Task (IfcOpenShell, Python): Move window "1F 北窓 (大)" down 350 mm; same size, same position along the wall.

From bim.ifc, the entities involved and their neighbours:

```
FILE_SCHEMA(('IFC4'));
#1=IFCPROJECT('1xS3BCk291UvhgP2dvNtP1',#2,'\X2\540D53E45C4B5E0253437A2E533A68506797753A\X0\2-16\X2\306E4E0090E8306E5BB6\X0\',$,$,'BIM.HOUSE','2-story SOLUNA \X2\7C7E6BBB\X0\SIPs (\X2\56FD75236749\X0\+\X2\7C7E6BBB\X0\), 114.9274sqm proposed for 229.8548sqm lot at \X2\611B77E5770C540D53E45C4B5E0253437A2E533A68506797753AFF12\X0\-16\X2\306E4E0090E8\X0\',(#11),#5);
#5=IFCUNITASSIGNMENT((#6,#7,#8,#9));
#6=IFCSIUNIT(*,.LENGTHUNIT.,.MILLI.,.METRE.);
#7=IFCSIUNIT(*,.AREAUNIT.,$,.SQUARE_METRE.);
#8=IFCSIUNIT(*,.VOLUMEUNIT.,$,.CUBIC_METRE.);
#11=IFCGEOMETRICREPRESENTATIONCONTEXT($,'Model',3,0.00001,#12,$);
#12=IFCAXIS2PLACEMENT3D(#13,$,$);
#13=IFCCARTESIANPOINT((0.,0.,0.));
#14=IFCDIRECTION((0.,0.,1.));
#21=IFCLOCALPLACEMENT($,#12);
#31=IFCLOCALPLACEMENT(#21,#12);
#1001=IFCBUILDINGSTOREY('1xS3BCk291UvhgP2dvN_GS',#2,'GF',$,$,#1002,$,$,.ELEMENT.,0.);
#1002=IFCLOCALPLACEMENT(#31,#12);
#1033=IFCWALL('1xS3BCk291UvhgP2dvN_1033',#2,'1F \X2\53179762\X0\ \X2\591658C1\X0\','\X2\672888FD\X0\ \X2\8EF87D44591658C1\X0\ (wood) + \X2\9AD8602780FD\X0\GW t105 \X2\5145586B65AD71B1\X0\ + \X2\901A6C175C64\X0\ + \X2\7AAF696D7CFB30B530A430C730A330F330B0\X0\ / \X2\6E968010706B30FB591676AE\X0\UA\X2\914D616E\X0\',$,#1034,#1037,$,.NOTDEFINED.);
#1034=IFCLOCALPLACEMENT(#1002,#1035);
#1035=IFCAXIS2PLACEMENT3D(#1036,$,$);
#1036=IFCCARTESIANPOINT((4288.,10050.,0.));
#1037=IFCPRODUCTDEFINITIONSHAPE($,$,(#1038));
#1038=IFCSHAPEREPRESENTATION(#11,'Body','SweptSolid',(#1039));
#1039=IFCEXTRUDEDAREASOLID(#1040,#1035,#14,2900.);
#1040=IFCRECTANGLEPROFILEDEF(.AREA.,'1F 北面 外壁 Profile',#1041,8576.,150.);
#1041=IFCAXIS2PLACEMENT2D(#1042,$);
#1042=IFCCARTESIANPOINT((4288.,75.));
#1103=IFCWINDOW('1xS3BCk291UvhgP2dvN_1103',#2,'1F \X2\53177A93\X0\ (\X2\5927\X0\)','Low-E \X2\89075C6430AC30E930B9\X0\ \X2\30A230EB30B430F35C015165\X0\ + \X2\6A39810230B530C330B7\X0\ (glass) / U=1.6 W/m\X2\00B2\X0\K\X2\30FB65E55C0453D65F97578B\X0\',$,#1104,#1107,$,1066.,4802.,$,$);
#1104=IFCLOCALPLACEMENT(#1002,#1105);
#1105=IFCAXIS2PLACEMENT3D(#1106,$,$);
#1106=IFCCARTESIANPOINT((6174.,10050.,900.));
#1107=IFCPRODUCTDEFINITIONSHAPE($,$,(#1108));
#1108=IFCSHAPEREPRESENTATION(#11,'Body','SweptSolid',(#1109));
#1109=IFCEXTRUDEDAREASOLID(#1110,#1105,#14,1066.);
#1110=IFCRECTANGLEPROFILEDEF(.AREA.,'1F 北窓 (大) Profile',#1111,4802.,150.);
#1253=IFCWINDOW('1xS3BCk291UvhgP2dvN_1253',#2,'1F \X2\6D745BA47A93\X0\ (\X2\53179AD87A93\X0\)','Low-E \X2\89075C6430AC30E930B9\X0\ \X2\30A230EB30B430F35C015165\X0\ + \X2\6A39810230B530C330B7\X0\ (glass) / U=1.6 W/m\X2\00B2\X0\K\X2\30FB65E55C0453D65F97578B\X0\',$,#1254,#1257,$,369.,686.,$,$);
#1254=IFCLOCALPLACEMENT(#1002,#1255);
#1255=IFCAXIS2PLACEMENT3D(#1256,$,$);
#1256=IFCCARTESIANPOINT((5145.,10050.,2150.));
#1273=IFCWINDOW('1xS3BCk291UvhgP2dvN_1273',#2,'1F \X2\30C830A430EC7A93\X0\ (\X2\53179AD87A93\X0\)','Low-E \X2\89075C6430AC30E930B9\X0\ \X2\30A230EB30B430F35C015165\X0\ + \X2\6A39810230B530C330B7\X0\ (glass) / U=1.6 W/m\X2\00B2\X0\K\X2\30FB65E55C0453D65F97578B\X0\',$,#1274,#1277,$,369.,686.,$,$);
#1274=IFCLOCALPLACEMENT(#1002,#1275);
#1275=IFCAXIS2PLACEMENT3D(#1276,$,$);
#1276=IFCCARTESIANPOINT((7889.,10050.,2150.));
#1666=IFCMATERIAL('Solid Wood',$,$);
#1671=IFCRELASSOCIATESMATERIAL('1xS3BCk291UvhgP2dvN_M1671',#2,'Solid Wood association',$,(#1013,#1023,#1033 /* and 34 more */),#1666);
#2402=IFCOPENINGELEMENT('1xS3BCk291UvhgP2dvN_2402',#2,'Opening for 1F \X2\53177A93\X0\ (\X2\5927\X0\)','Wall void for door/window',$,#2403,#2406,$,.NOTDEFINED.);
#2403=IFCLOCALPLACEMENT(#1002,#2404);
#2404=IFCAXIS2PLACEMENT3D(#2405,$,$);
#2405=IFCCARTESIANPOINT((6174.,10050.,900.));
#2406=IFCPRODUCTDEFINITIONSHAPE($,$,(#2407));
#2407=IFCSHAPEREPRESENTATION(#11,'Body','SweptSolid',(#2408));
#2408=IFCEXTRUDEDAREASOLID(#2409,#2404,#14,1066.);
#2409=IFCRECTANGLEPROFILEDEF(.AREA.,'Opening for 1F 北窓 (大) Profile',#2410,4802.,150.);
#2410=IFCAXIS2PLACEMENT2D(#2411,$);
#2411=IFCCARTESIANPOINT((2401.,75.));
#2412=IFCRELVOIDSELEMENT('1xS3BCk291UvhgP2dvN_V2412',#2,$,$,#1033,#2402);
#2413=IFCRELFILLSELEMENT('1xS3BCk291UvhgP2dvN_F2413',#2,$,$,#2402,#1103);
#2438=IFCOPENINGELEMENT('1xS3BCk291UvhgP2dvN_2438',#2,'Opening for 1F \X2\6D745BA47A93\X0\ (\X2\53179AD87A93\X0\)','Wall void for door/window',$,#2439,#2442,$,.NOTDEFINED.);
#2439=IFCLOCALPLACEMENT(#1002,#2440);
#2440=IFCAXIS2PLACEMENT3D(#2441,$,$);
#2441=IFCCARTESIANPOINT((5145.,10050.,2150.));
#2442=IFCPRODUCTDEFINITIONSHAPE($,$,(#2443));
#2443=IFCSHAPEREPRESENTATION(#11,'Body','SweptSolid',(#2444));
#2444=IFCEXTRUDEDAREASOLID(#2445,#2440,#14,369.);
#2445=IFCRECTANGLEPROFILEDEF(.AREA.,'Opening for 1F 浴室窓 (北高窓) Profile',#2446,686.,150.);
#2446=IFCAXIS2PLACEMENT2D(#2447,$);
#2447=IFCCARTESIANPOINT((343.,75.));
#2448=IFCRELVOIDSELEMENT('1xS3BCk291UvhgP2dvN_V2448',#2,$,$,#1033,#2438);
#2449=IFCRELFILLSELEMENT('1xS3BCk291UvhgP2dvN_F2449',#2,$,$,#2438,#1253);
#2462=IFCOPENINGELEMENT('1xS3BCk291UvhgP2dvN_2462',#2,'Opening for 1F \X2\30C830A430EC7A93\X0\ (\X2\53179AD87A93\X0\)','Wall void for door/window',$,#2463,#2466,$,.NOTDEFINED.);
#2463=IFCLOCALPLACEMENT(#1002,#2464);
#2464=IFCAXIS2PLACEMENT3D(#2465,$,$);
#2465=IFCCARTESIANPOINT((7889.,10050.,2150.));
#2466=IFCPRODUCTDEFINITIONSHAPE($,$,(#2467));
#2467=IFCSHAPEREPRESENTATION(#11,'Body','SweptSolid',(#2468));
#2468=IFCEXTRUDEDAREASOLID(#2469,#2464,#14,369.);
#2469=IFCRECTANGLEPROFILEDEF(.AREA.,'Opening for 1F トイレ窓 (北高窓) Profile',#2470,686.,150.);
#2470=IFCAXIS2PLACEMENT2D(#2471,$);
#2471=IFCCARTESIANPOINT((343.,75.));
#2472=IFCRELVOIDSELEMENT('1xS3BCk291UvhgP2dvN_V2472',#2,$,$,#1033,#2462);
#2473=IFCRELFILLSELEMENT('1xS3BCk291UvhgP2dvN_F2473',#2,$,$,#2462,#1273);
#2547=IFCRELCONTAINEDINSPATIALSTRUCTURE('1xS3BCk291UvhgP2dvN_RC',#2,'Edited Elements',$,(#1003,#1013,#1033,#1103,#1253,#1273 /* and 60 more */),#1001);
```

```python
import numpy as np
import ifcopenshell
import ifcopenshell.api.geometry
import ifcopenshell.util.placement
import ifcopenshell.util.unit

model = ifcopenshell.open("bim.ifc")
unit_scale = ifcopenshell.util.unit.calculate_unit_scale(model)

window = model.by_id(1103)
opening = window.FillsVoids[0].RelatingOpeningElement
dz = -0.35 / unit_scale

shift = np.array([0.0, 0.0, dz])
# The window is not placed relative to its opening, so move both.
for product in (opening, window):
    matrix = ifcopenshell.util.placement.get_local_placement(product.ObjectPlacement)
    matrix[:3, 3] += shift
    ifcopenshell.api.geometry.edit_object_placement(model, product=product, matrix=matrix, is_si=False)

print(f"moved by {dz * unit_scale:+.3f} m")

model.write("bim_updated.ifc")
```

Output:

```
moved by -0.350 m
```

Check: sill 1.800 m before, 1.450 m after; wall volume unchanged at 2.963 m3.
